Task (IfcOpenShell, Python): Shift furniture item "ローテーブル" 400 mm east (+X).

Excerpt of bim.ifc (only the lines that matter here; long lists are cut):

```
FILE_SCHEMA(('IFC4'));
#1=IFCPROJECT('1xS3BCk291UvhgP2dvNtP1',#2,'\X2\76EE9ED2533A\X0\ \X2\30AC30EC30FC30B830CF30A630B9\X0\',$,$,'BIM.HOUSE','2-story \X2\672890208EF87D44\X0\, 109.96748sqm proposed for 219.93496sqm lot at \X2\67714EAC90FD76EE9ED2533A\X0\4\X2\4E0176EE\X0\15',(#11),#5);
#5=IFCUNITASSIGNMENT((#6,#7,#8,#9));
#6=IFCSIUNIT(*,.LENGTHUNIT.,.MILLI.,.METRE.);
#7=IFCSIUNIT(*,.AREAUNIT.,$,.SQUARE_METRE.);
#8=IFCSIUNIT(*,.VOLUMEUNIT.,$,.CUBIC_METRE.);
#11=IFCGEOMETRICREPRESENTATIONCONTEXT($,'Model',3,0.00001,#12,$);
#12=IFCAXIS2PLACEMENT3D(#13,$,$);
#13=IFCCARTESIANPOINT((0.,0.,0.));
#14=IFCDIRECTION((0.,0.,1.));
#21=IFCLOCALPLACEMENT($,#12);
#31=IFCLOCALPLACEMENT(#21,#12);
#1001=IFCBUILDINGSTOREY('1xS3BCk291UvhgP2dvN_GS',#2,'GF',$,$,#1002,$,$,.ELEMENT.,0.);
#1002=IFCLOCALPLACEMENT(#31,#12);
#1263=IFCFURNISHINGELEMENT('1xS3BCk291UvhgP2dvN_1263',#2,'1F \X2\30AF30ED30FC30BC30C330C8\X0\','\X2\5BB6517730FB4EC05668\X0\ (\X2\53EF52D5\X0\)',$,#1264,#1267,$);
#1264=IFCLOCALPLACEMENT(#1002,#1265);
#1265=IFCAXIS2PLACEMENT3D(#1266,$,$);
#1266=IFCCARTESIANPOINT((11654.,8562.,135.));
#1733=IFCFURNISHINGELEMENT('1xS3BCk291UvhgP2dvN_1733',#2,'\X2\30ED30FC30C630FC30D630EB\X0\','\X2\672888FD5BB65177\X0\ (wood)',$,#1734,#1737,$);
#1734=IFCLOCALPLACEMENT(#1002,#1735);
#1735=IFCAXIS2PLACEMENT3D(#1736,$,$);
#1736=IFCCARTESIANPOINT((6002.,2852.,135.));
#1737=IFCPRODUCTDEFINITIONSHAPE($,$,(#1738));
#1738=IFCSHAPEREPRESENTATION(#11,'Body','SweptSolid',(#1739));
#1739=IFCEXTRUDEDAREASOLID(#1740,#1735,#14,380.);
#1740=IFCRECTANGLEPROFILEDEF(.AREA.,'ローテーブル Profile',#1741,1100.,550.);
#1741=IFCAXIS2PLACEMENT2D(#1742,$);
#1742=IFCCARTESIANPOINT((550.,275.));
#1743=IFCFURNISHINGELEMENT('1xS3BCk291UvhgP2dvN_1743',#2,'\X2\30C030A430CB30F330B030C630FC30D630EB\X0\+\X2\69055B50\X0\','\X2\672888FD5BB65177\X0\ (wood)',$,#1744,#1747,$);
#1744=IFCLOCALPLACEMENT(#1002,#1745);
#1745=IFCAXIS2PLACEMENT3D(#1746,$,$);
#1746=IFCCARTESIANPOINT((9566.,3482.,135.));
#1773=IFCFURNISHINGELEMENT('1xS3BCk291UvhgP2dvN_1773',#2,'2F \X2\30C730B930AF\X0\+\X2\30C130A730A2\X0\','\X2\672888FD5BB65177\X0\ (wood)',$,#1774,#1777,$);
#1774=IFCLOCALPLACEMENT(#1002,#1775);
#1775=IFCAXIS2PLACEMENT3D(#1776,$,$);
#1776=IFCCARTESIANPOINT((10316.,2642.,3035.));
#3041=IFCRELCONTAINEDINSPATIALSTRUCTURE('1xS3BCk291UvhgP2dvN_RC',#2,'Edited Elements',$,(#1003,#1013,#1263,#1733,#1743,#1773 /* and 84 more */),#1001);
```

```python
import ifcopenshell
import ifcopenshell.api.geometry
import ifcopenshell.util.placement

model = ifcopenshell.open("bim.ifc")

item = model.by_id(1733)
matrix = ifcopenshell.util.placement.get_local_placement(item.ObjectPlacement)
matrix[0, 3] += 400.0
ifcopenshell.api.geometry.edit_object_placement(model, product=item, matrix=matrix, is_si=False)

print(ifcopenshell.util.placement.get_local_placement(item.ObjectPlacement).round(3) + 0.0)

model.write("bim_updated.ifc")
```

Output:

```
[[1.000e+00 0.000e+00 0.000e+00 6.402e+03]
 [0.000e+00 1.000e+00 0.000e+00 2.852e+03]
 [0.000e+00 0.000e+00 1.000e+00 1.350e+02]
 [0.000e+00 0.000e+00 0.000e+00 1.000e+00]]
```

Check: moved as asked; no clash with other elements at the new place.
